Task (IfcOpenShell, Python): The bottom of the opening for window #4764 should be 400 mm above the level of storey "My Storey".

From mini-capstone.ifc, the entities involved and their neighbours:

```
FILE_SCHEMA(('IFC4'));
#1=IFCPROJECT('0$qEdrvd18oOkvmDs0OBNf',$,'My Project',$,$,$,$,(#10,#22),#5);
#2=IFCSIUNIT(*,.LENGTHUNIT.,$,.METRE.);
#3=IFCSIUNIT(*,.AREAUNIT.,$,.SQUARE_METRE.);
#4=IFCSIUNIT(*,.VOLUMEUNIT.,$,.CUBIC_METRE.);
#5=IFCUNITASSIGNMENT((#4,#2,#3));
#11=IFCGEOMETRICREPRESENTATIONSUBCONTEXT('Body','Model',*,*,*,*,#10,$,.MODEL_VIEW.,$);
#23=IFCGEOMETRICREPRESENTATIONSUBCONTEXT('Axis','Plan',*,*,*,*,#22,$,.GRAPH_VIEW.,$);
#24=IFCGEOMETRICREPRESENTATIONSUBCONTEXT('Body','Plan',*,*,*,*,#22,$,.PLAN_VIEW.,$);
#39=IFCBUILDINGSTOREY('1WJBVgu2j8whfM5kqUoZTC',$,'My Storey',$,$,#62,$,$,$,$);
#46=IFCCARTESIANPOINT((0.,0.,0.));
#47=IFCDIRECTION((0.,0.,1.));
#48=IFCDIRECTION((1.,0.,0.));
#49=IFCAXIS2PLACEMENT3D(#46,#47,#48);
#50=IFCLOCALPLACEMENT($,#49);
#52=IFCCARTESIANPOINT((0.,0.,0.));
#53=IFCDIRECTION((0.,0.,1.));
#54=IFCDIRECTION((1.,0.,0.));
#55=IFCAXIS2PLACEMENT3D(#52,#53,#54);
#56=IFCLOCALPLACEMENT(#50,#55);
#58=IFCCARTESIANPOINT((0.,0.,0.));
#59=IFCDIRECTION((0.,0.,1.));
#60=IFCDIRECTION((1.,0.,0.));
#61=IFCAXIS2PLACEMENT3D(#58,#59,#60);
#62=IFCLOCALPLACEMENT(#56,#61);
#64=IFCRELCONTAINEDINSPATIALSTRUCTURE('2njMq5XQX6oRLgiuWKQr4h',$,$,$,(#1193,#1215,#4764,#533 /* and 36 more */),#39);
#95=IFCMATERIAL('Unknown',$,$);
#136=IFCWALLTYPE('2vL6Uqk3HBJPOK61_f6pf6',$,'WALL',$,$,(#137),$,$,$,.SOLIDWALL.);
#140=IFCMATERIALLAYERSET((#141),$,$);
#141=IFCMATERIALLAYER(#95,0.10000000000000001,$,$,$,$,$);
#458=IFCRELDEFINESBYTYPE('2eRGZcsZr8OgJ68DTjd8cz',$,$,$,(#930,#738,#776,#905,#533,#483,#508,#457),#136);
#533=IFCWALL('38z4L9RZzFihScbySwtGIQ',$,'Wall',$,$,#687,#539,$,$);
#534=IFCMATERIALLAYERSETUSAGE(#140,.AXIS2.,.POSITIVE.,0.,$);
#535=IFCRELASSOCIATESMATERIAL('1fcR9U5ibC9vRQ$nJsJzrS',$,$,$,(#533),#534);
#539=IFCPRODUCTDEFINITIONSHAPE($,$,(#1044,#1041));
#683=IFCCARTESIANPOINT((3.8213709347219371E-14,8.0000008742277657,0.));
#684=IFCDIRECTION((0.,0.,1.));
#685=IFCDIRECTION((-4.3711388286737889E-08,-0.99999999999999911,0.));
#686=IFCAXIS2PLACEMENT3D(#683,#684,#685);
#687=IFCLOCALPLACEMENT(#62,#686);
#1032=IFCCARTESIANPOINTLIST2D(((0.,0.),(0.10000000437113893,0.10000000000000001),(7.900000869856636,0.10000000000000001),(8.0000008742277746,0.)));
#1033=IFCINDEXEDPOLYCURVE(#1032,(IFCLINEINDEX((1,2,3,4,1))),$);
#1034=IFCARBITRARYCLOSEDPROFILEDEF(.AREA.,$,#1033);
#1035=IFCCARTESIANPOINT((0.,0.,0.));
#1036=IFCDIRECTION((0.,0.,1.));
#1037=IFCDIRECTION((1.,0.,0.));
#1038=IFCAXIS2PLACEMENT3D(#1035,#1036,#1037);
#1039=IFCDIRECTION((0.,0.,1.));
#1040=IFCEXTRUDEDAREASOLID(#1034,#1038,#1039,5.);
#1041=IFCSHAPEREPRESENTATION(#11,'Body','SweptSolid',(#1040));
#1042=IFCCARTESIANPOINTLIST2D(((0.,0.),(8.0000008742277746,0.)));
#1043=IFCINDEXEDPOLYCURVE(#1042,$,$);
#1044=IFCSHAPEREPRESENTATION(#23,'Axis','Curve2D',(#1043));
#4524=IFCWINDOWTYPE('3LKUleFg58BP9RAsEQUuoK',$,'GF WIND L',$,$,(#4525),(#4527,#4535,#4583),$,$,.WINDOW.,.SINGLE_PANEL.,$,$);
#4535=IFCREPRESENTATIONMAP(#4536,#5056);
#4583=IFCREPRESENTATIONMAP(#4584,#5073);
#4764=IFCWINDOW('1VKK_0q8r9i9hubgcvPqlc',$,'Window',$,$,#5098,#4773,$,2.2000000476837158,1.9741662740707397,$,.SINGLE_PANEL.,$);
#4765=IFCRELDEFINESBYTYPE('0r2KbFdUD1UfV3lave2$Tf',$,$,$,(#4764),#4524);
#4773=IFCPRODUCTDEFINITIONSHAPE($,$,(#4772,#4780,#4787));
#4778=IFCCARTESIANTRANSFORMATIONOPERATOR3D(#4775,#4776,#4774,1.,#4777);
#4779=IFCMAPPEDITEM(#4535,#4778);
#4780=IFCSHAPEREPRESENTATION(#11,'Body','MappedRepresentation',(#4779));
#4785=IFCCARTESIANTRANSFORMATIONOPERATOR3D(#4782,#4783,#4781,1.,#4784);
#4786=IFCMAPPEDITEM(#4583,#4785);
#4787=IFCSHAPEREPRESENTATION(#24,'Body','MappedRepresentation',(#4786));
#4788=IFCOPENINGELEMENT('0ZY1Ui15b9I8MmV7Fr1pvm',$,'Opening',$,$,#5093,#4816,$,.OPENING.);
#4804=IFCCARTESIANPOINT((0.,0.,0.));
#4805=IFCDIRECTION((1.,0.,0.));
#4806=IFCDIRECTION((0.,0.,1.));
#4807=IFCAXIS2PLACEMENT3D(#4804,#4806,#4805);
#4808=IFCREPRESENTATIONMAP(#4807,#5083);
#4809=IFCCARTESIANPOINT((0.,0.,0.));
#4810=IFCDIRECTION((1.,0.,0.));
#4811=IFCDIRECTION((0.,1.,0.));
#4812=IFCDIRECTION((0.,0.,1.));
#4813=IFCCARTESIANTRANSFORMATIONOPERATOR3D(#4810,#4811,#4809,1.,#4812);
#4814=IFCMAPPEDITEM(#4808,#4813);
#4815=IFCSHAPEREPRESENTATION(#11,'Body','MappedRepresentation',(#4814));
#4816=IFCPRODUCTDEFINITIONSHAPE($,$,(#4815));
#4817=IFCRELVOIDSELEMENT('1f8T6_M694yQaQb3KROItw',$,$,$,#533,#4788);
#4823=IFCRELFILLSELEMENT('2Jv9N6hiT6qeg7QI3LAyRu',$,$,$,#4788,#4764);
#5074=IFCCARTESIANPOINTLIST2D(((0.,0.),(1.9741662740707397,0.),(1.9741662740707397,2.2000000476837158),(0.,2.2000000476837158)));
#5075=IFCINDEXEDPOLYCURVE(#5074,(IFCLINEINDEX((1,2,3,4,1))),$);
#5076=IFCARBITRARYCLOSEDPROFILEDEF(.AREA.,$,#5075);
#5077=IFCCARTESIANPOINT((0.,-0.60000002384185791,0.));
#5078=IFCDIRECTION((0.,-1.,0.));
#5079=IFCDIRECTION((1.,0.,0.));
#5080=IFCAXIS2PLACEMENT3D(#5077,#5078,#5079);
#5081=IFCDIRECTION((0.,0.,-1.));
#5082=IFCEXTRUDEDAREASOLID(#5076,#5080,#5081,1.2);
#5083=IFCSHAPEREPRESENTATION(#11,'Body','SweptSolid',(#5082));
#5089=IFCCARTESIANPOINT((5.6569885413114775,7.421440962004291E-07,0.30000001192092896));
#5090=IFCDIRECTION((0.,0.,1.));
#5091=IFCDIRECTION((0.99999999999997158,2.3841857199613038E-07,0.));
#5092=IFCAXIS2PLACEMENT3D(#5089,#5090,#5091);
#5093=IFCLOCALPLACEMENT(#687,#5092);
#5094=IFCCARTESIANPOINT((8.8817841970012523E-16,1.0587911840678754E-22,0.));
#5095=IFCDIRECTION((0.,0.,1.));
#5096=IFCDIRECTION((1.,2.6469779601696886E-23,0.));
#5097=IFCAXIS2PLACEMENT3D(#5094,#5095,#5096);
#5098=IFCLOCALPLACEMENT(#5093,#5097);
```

```python
import numpy as np
import ifcopenshell
import ifcopenshell.api.geometry
import ifcopenshell.geom
import ifcopenshell.util.element
import ifcopenshell.util.placement
import ifcopenshell.util.shape
import ifcopenshell.util.unit

model = ifcopenshell.open("mini-capstone.ifc")
unit_scale = ifcopenshell.util.unit.calculate_unit_scale(model)

window = model.by_guid("1VKK_0q8r9i9hubgcvPqlc")
opening = window.FillsVoids[0].RelatingOpeningElement
storey = ifcopenshell.util.element.get_container(window, ifc_class="IfcBuildingStorey")
level = ifcopenshell.util.placement.get_local_placement(storey.ObjectPlacement)[2, 3]

# The opening's origin need not be at the sill, so measure its lowest point.
shape = ifcopenshell.geom.create_shape(ifcopenshell.geom.settings(), opening)
bottom = ifcopenshell.util.shape.get_shape_bottom_elevation(shape, shape.geometry) / unit_scale
dz = level + 0.4 / unit_scale - bottom

shift = np.array([0.0, 0.0, dz])
# The window is placed relative to its opening, so it follows when the opening moves.
matrix = ifcopenshell.util.placement.get_local_placement(opening.ObjectPlacement)
matrix[:3, 3] += shift
ifcopenshell.api.geometry.edit_object_placement(
    model, product=opening, matrix=matrix, is_si=False, should_transform_children=True
)

print(f"moved by {dz * unit_scale:+.3f} m")

model.write("mini-capstone_rev.ifc")
```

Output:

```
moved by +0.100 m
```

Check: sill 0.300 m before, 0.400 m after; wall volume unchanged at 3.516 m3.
